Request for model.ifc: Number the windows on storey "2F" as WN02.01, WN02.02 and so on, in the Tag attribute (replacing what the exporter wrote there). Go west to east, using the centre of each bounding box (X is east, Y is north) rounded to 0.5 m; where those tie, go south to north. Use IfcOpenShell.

First a look at what the model holds.

```python
import ifcopenshell
import ifcopenshell.util.element
import ifcopenshell.util.placement

model = ifcopenshell.open("model.ifc")
print(model.schema)
storey = next(s for s in model.by_type("IfcBuildingStorey") if s.Name == "2F")
windows = [e for e in ifcopenshell.util.element.get_decomposition(storey) if e.is_a("IfcWindow")]
for e in sorted(windows, key=lambda e: e.id()):
    origin = ifcopenshell.util.placement.get_local_placement(e.ObjectPlacement)[:3, 3]
    print(e.id(), e.Tag, e.Name, origin.round(2) + 0.0, sep=" | ")
```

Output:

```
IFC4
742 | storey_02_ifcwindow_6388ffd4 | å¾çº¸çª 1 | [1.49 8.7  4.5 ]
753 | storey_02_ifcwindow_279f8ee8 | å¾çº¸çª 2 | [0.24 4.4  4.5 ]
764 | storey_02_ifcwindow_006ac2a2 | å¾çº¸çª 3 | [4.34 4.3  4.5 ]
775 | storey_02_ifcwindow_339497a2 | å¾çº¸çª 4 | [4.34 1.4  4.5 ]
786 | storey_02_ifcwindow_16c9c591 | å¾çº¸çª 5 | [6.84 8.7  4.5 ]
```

```python
import ifcopenshell
import ifcopenshell.geom
import ifcopenshell.util.element
import ifcopenshell.util.shape

model = ifcopenshell.open("model.ifc")
settings = ifcopenshell.geom.settings()
settings.set("use-world-coords", True)


def centre(element):
    shape = ifcopenshell.geom.create_shape(settings, element)
    return ifcopenshell.util.shape.get_bbox_centroid(shape.geometry)


storey = next(s for s in model.by_type("IfcBuildingStorey") if s.Name == "2F")
windows = [e for e in ifcopenshell.util.element.get_decomposition(storey) if e.is_a("IfcWindow")]

# Insertion points can sit at a corner or the storey origin, so sort by the geometry (in metres).
centres = {e: centre(e) for e in windows}
windows.sort(key=lambda e: (round(centres[e][0] / 0.5), centres[e][1]))

for i, e in enumerate(windows, start=1):
    number = f"WN02.{i:02d}"
    e.Tag = number
    print(e.id(), number)

model.write("model-out.ifc")
```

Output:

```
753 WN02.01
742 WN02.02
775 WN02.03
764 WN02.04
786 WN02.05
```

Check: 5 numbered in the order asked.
